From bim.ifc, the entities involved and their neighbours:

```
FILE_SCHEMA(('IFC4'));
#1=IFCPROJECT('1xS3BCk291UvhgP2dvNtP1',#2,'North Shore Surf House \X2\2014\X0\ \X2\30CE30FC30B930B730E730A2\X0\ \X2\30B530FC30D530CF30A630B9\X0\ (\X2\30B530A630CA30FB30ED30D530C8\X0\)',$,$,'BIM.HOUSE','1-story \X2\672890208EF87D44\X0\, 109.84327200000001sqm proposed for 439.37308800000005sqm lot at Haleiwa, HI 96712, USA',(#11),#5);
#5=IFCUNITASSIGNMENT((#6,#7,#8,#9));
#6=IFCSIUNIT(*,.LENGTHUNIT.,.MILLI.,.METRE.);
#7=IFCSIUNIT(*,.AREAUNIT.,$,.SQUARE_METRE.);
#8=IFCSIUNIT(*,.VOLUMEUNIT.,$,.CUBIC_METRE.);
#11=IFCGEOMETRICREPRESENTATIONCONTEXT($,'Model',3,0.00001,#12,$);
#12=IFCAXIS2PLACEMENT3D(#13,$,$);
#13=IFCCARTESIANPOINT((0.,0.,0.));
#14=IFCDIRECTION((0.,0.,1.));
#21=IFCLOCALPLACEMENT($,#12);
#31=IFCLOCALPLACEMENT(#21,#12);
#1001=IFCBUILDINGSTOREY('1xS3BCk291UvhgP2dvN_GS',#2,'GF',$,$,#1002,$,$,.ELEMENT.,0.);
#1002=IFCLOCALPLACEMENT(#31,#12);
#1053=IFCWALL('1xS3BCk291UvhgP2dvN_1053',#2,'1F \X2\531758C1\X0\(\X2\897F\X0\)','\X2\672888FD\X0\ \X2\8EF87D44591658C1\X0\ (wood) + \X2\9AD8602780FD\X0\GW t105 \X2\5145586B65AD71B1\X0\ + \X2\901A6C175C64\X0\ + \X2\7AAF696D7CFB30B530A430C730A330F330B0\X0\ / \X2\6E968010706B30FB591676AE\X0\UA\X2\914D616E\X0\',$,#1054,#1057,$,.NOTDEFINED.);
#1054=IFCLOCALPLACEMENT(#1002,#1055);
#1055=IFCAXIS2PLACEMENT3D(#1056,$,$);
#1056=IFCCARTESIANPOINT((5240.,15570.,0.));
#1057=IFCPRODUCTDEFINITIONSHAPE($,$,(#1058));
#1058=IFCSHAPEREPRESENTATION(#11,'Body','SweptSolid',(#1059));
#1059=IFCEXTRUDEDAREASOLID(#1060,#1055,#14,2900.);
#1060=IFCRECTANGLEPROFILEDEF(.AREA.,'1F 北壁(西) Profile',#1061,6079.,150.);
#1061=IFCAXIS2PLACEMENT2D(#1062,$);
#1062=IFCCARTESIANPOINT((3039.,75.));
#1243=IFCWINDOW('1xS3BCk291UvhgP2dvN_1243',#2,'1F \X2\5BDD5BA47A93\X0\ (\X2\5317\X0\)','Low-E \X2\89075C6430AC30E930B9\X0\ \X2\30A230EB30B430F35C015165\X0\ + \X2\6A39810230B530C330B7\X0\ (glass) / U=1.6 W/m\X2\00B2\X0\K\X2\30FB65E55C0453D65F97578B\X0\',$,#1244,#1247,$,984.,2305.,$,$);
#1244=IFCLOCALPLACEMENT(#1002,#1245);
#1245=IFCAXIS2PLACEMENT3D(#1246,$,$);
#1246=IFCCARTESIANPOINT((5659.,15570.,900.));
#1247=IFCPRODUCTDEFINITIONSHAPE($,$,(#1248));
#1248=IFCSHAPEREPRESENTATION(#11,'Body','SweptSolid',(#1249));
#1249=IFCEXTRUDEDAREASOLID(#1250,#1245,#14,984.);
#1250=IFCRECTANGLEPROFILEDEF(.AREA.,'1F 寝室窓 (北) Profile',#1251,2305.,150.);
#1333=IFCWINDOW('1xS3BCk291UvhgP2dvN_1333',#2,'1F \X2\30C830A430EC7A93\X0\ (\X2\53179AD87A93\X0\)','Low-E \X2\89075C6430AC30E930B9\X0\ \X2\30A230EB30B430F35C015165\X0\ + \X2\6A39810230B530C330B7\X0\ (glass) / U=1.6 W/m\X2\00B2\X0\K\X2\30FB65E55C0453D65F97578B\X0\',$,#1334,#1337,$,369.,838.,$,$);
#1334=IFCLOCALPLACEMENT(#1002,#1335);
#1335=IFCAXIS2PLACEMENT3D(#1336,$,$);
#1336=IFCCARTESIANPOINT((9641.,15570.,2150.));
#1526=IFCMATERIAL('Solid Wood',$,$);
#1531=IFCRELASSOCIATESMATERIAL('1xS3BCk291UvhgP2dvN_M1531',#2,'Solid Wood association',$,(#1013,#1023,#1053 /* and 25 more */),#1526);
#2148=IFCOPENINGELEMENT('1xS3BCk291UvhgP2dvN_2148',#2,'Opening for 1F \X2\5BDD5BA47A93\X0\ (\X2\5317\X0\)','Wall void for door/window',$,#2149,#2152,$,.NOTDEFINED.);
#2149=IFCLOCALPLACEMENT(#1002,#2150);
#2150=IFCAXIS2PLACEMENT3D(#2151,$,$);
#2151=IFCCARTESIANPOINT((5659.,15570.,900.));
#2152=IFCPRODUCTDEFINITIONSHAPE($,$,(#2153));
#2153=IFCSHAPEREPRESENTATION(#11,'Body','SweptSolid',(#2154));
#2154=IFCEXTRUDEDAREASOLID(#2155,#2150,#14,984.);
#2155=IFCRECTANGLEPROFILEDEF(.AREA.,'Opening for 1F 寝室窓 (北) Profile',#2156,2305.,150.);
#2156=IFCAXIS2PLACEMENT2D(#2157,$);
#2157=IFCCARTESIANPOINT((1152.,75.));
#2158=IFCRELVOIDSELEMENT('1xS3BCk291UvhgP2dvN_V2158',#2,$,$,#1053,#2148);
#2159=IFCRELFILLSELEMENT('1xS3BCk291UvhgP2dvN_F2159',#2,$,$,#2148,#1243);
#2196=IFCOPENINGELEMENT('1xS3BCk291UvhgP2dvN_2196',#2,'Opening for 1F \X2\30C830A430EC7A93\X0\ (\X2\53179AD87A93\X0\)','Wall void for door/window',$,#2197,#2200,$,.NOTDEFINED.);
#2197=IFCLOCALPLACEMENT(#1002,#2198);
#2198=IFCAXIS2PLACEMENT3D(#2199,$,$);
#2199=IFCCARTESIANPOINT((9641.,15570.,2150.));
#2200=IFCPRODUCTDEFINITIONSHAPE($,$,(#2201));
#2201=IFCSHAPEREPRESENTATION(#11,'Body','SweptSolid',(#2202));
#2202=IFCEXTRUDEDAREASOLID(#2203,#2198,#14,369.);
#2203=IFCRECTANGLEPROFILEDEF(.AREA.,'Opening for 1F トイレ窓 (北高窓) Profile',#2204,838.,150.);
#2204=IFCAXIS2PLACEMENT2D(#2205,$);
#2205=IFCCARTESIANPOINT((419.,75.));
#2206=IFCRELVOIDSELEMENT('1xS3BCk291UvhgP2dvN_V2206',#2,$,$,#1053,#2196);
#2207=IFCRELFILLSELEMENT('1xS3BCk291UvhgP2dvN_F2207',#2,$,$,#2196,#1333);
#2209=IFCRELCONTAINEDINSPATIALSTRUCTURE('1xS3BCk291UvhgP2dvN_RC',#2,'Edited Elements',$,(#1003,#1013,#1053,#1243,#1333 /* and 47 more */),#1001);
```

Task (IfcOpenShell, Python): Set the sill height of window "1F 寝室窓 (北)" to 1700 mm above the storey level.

```python
import numpy as np
import ifcopenshell
import ifcopenshell.api.geometry
import ifcopenshell.geom
import ifcopenshell.util.element
import ifcopenshell.util.placement
import ifcopenshell.util.shape
import ifcopenshell.util.unit

model = ifcopenshell.open("bim.ifc")
unit_scale = ifcopenshell.util.unit.calculate_unit_scale(model)

window = model.by_guid("1xS3BCk291UvhgP2dvN_1243")
opening = window.FillsVoids[0].RelatingOpeningElement
storey = ifcopenshell.util.element.get_container(window, ifc_class="IfcBuildingStorey")
level = ifcopenshell.util.placement.get_local_placement(storey.ObjectPlacement)[2, 3]

# The opening's origin need not be at the sill, so measure its lowest point.
shape = ifcopenshell.geom.create_shape(ifcopenshell.geom.settings(), opening)
bottom = ifcopenshell.util.shape.get_shape_bottom_elevation(shape, shape.geometry) / unit_scale
dz = level + 1.7 / unit_scale - bottom

shift = np.array([0.0, 0.0, dz])
# The window is not placed relative to its opening, so move both.
for product in (opening, window):
    matrix = ifcopenshell.util.placement.get_local_placement(product.ObjectPlacement)
    matrix[:3, 3] += shift
    ifcopenshell.api.geometry.edit_object_placement(model, product=product, matrix=matrix, is_si=False)

print(f"moved by {dz * unit_scale:+.3f} m")

model.write("bim_updated.ifc")
```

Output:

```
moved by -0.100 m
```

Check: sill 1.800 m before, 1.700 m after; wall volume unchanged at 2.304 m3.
